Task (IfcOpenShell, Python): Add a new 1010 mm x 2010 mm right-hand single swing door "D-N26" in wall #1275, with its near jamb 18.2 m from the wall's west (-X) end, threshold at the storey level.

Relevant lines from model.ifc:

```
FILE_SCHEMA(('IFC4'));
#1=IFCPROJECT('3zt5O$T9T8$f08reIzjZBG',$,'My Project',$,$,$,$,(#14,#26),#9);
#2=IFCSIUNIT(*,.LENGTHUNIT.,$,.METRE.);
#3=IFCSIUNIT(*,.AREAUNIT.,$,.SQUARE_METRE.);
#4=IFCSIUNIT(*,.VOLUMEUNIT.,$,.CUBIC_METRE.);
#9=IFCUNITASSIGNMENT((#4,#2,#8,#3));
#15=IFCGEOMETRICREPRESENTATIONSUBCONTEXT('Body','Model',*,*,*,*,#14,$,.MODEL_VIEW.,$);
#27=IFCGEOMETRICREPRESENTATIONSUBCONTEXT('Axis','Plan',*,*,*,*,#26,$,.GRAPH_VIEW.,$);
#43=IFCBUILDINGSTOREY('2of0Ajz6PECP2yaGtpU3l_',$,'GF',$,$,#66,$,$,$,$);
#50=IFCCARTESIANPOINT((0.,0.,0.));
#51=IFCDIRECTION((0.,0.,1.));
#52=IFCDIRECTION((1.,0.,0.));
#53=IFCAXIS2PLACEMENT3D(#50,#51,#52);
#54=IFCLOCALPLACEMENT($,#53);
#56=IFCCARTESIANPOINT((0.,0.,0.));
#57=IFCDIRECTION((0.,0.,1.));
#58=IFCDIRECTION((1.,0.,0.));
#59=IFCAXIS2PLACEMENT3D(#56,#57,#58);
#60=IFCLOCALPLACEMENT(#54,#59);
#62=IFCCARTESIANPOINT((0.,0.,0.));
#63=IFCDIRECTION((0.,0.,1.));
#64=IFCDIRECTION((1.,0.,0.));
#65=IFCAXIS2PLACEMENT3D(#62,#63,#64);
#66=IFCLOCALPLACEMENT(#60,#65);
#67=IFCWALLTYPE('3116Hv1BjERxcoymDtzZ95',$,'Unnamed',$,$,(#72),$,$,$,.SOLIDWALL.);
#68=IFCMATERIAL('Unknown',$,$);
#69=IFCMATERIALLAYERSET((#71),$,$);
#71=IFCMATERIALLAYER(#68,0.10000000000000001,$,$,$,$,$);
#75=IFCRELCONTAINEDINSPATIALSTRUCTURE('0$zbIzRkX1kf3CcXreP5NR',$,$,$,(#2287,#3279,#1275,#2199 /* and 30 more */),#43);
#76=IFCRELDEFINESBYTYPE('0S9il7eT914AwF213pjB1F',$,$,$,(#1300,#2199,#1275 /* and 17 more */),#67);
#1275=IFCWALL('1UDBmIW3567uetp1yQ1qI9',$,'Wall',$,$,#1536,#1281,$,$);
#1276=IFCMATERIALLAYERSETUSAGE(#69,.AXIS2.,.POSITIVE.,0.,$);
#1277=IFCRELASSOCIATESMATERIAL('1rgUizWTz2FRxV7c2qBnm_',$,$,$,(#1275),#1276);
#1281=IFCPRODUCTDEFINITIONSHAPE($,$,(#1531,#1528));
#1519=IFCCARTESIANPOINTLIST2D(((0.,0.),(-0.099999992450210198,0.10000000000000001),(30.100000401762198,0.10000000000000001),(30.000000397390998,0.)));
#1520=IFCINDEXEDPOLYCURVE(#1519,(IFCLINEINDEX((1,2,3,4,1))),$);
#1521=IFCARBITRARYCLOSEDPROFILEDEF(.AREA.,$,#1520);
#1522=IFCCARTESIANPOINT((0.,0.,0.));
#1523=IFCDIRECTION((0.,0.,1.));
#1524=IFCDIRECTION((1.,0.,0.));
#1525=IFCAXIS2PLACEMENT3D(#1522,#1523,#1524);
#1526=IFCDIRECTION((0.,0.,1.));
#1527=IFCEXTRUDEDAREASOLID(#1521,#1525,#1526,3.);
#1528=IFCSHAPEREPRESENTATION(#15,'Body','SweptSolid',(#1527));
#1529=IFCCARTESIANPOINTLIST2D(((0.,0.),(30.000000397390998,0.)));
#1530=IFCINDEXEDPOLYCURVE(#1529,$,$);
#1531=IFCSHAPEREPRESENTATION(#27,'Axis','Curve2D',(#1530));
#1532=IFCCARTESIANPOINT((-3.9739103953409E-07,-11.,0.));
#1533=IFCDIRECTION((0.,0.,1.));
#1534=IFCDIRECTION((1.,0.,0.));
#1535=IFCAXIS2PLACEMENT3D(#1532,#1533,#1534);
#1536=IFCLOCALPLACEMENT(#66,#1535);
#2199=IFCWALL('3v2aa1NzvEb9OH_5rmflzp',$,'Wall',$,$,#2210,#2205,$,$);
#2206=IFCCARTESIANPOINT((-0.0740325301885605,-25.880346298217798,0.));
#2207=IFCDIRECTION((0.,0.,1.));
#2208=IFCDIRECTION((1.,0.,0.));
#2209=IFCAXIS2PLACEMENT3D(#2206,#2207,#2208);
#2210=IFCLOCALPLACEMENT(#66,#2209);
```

```python
import numpy as np
import ifcopenshell
import ifcopenshell.api.feature
import ifcopenshell.api.geometry
import ifcopenshell.api.root
import ifcopenshell.api.spatial
import ifcopenshell.geom
import ifcopenshell.util.element
import ifcopenshell.util.placement
import ifcopenshell.util.representation
import ifcopenshell.util.shape
import ifcopenshell.util.unit

model = ifcopenshell.open("model.ifc")
unit_scale = ifcopenshell.util.unit.calculate_unit_scale(model)
settings = ifcopenshell.geom.settings()


def volume(element):
    """Net volume in cubic metres, openings subtracted."""
    shape = ifcopenshell.geom.create_shape(settings, element)
    return ifcopenshell.util.shape.get_volume(shape.geometry)


wall = model.by_id(1275)
storey = ifcopenshell.util.element.get_container(wall, ifc_class="IfcBuildingStorey")
context = ifcopenshell.util.representation.get_context(model, "Model", "Body", "MODEL_VIEW")
before = volume(wall)

width, height, from_end, sill = 1.01, 2.01, 18.2, 0.0  # metres

# The wall runs along its own X axis, and the end named is its -X end.
wall_shape = ifcopenshell.geom.create_shape(settings, wall)
x, y, z = ifcopenshell.util.shape.get_vertices(wall_shape.geometry).T
start = x.min() + from_end
face, thickness = float(y.min()), float(y.max() - y.min())
wall_matrix = ifcopenshell.util.placement.get_local_placement(wall.ObjectPlacement)
level = ifcopenshell.util.placement.get_local_placement(storey.ObjectPlacement)[2, 3]


def in_wall(x, y):
    """Placement at x, y metres in the wall's axes, at sill height."""
    matrix = wall_matrix.copy()
    matrix[:, 3] = wall_matrix @ np.array([x / unit_scale, y / unit_scale, 0.0, 1.0])
    matrix[2, 3] = level + sill / unit_scale
    return matrix


# Opening: a box that overshoots both wall faces by 50 mm.
opening = ifcopenshell.api.root.create_entity(model, ifc_class="IfcOpeningElement", predefined_type="OPENING")
box = ifcopenshell.api.geometry.add_wall_representation(
    model, context=context, length=width, height=height, thickness=thickness + 0.1
)
ifcopenshell.api.geometry.assign_representation(model, product=opening, representation=box)
ifcopenshell.api.geometry.edit_object_placement(model, product=opening, matrix=in_wall(start, face - 0.05), is_si=False)
ifcopenshell.api.feature.add_feature(model, feature=opening, element=wall)

door = ifcopenshell.api.root.create_entity(model, ifc_class="IfcDoor", name="D-N26", predefined_type="DOOR")
door.OverallWidth, door.OverallHeight = width / unit_scale, height / unit_scale
door.OperationType = "SINGLE_SWING_RIGHT"
body = ifcopenshell.api.geometry.add_door_representation(
    model,
    context=context,
    overall_width=door.OverallWidth,
    overall_height=door.OverallHeight,
    operation_type="SINGLE_SWING_RIGHT",
    lining_properties={"LiningDepth": thickness / unit_scale, "ThresholdDepth": thickness / unit_scale},
)
ifcopenshell.api.geometry.assign_representation(model, product=door, representation=body)
ifcopenshell.api.spatial.assign_container(model, products=[door], relating_structure=storey)
ifcopenshell.api.feature.add_filling(model, opening=opening, element=door)

# The lining spans the wall, so the door starts at the wall face.
ifcopenshell.api.geometry.edit_object_placement(model, product=door, matrix=in_wall(start, face), is_si=False)

after = volume(wall)

print(f"wall volume {before:.3f} -> {after:.3f} m3")

model.write("model_edited.ifc")
```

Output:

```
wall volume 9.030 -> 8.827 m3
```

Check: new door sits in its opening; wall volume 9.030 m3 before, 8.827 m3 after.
